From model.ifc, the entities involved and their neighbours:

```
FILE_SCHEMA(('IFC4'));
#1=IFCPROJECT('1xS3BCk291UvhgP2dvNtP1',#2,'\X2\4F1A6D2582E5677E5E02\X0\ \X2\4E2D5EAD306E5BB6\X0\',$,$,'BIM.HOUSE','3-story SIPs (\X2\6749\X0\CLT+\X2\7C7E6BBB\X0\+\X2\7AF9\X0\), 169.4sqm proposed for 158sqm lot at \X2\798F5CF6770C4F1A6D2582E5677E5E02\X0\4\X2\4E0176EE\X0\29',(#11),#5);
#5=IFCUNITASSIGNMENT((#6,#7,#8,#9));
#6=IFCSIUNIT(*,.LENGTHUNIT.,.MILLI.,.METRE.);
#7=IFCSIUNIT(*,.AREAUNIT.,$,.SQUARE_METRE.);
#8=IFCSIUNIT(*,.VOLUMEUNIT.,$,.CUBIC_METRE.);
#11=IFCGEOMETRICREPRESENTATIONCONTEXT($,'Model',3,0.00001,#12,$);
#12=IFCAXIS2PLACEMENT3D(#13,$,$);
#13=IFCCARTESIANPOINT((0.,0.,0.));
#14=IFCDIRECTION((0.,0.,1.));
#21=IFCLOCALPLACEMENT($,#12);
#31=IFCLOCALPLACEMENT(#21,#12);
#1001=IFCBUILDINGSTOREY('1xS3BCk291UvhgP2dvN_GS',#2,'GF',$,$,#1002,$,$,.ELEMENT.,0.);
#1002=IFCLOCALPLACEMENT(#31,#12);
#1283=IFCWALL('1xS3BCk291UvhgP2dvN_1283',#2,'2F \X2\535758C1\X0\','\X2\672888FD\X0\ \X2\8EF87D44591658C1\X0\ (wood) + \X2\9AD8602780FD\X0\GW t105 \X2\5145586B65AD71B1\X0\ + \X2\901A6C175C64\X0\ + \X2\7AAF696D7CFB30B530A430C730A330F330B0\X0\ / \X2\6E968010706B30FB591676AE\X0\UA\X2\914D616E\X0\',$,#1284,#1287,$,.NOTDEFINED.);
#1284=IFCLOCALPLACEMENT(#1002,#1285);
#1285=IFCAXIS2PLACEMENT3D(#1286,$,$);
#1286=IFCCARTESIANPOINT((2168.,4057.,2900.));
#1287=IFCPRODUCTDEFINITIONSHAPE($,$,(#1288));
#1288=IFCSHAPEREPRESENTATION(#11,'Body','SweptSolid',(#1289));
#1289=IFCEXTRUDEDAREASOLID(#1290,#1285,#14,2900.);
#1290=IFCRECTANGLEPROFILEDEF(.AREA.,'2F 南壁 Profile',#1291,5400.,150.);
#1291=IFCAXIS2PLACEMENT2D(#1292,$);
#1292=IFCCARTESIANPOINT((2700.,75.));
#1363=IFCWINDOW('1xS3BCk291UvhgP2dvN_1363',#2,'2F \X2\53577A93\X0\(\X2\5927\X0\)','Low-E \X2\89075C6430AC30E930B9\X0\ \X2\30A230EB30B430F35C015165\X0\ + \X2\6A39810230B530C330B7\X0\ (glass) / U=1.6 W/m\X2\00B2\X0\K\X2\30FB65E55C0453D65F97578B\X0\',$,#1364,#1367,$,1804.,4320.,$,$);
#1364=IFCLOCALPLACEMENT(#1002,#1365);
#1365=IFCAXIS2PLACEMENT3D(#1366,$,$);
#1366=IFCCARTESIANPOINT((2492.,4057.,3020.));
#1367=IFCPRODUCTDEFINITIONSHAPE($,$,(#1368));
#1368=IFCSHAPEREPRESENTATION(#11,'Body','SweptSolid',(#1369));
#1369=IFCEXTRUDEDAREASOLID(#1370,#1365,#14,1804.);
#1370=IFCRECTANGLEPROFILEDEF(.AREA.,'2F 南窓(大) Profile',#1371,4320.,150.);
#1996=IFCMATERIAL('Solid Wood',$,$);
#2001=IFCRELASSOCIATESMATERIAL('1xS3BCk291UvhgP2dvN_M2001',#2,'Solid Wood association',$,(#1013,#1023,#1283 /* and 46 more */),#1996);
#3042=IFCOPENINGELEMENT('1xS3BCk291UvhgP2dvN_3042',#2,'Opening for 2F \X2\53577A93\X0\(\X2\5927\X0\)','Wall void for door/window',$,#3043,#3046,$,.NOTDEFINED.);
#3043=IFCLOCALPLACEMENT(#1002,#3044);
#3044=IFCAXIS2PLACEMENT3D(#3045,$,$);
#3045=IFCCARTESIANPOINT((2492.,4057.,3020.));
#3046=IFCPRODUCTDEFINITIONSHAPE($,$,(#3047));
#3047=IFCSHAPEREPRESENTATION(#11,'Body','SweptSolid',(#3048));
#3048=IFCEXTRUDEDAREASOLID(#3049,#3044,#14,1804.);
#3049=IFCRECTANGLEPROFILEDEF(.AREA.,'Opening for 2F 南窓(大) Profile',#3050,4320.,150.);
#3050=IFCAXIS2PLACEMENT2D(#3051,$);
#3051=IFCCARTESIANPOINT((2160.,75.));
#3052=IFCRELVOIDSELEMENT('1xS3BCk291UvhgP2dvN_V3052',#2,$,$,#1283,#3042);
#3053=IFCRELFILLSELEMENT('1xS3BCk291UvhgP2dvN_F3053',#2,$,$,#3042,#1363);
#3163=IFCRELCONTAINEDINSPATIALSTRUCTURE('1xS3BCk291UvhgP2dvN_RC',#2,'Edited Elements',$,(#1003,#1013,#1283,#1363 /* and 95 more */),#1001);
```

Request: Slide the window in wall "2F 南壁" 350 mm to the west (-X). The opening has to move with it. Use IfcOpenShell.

```python
import ifcopenshell
import ifcopenshell.api.geometry
import ifcopenshell.util.placement

model = ifcopenshell.open("model.ifc")

window = model.by_id(1363)
opening = window.FillsVoids[0].RelatingOpeningElement
wall = opening.VoidsElements[0].RelatingBuildingElement

wall_matrix = ifcopenshell.util.placement.get_local_placement(wall.ObjectPlacement)
shift = wall_matrix[:3, 0] * -350.0
before = ifcopenshell.util.placement.get_local_placement(window.ObjectPlacement)[:3, 3].copy()

# The window is not placed relative to its opening, so move both.
for product in (opening, window):
    matrix = ifcopenshell.util.placement.get_local_placement(product.ObjectPlacement)
    matrix[:3, 3] += shift
    ifcopenshell.api.geometry.edit_object_placement(model, product=product, matrix=matrix, is_si=False)

after = ifcopenshell.util.placement.get_local_placement(window.ObjectPlacement)[:3, 3]
print("window moved by", (after - before).round(3) + 0.0)

model.write("model-out.ifc")
```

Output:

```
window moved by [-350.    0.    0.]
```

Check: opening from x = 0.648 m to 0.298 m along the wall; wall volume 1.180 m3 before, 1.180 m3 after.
